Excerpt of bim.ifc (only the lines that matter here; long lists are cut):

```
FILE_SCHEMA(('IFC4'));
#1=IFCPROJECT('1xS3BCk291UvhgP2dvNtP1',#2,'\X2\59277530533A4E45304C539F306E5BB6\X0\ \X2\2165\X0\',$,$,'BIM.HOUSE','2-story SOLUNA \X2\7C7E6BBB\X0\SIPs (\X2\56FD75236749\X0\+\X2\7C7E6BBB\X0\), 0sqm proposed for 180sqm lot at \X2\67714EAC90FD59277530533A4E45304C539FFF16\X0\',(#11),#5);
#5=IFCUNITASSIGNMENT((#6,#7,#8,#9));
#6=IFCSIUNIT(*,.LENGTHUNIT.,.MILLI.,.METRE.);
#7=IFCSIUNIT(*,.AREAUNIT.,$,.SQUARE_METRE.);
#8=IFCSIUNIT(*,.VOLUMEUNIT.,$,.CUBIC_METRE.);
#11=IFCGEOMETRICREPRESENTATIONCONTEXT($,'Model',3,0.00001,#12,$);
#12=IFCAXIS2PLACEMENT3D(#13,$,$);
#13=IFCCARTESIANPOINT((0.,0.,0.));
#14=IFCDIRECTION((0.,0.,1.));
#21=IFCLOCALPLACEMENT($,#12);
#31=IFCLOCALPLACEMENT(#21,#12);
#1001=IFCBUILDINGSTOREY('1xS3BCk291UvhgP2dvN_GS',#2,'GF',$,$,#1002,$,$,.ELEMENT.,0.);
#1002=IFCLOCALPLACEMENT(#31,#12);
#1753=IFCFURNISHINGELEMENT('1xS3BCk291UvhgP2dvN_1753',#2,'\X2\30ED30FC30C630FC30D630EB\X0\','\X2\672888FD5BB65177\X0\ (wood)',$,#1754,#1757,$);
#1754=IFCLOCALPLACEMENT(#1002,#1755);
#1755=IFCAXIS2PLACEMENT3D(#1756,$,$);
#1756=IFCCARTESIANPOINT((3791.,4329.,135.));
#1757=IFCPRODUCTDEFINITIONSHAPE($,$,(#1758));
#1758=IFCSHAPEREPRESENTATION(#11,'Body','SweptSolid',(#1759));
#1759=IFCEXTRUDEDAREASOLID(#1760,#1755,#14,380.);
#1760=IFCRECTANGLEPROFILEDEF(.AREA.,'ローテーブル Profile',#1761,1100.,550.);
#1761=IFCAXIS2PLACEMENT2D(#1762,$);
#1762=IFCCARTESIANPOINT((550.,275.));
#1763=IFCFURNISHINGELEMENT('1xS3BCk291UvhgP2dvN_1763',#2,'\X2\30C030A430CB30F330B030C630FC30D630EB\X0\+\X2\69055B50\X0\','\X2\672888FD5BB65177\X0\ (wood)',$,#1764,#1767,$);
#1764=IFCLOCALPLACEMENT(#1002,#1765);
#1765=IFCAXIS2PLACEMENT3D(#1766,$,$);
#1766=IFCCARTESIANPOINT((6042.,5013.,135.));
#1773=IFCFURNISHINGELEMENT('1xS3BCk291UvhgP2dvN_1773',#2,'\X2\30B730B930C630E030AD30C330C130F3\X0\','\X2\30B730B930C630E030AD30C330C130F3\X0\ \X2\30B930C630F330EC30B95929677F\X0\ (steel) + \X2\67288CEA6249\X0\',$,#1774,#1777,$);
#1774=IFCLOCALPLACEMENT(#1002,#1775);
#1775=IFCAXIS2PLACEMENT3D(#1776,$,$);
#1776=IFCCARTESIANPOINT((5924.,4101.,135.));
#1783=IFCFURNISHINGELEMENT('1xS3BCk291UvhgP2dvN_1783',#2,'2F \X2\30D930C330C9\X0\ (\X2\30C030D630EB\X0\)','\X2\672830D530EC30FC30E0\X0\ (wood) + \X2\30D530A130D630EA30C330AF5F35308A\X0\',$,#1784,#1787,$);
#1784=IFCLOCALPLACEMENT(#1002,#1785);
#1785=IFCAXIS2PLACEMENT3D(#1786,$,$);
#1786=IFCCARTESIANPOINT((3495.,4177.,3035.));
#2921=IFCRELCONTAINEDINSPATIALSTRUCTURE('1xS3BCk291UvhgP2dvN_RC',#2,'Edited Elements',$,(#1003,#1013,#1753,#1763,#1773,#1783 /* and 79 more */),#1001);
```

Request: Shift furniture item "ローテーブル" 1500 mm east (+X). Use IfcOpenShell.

```python
import ifcopenshell
import ifcopenshell.api.geometry
import ifcopenshell.util.placement
import ifcopenshell.util.unit

model = ifcopenshell.open("bim.ifc")
unit_scale = ifcopenshell.util.unit.calculate_unit_scale(model)

item = model.by_guid("1xS3BCk291UvhgP2dvN_1753")
matrix = ifcopenshell.util.placement.get_local_placement(item.ObjectPlacement)
matrix[0, 3] += 1.5 / unit_scale
ifcopenshell.api.geometry.edit_object_placement(model, product=item, matrix=matrix, is_si=False)

print(ifcopenshell.util.placement.get_local_placement(item.ObjectPlacement).round(3) + 0.0)

model.write("bim_updated.ifc")
```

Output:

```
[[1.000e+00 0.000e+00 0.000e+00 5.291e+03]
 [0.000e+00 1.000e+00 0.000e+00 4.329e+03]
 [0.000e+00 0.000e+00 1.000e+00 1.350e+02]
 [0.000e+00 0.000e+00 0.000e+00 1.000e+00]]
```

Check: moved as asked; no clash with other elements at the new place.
